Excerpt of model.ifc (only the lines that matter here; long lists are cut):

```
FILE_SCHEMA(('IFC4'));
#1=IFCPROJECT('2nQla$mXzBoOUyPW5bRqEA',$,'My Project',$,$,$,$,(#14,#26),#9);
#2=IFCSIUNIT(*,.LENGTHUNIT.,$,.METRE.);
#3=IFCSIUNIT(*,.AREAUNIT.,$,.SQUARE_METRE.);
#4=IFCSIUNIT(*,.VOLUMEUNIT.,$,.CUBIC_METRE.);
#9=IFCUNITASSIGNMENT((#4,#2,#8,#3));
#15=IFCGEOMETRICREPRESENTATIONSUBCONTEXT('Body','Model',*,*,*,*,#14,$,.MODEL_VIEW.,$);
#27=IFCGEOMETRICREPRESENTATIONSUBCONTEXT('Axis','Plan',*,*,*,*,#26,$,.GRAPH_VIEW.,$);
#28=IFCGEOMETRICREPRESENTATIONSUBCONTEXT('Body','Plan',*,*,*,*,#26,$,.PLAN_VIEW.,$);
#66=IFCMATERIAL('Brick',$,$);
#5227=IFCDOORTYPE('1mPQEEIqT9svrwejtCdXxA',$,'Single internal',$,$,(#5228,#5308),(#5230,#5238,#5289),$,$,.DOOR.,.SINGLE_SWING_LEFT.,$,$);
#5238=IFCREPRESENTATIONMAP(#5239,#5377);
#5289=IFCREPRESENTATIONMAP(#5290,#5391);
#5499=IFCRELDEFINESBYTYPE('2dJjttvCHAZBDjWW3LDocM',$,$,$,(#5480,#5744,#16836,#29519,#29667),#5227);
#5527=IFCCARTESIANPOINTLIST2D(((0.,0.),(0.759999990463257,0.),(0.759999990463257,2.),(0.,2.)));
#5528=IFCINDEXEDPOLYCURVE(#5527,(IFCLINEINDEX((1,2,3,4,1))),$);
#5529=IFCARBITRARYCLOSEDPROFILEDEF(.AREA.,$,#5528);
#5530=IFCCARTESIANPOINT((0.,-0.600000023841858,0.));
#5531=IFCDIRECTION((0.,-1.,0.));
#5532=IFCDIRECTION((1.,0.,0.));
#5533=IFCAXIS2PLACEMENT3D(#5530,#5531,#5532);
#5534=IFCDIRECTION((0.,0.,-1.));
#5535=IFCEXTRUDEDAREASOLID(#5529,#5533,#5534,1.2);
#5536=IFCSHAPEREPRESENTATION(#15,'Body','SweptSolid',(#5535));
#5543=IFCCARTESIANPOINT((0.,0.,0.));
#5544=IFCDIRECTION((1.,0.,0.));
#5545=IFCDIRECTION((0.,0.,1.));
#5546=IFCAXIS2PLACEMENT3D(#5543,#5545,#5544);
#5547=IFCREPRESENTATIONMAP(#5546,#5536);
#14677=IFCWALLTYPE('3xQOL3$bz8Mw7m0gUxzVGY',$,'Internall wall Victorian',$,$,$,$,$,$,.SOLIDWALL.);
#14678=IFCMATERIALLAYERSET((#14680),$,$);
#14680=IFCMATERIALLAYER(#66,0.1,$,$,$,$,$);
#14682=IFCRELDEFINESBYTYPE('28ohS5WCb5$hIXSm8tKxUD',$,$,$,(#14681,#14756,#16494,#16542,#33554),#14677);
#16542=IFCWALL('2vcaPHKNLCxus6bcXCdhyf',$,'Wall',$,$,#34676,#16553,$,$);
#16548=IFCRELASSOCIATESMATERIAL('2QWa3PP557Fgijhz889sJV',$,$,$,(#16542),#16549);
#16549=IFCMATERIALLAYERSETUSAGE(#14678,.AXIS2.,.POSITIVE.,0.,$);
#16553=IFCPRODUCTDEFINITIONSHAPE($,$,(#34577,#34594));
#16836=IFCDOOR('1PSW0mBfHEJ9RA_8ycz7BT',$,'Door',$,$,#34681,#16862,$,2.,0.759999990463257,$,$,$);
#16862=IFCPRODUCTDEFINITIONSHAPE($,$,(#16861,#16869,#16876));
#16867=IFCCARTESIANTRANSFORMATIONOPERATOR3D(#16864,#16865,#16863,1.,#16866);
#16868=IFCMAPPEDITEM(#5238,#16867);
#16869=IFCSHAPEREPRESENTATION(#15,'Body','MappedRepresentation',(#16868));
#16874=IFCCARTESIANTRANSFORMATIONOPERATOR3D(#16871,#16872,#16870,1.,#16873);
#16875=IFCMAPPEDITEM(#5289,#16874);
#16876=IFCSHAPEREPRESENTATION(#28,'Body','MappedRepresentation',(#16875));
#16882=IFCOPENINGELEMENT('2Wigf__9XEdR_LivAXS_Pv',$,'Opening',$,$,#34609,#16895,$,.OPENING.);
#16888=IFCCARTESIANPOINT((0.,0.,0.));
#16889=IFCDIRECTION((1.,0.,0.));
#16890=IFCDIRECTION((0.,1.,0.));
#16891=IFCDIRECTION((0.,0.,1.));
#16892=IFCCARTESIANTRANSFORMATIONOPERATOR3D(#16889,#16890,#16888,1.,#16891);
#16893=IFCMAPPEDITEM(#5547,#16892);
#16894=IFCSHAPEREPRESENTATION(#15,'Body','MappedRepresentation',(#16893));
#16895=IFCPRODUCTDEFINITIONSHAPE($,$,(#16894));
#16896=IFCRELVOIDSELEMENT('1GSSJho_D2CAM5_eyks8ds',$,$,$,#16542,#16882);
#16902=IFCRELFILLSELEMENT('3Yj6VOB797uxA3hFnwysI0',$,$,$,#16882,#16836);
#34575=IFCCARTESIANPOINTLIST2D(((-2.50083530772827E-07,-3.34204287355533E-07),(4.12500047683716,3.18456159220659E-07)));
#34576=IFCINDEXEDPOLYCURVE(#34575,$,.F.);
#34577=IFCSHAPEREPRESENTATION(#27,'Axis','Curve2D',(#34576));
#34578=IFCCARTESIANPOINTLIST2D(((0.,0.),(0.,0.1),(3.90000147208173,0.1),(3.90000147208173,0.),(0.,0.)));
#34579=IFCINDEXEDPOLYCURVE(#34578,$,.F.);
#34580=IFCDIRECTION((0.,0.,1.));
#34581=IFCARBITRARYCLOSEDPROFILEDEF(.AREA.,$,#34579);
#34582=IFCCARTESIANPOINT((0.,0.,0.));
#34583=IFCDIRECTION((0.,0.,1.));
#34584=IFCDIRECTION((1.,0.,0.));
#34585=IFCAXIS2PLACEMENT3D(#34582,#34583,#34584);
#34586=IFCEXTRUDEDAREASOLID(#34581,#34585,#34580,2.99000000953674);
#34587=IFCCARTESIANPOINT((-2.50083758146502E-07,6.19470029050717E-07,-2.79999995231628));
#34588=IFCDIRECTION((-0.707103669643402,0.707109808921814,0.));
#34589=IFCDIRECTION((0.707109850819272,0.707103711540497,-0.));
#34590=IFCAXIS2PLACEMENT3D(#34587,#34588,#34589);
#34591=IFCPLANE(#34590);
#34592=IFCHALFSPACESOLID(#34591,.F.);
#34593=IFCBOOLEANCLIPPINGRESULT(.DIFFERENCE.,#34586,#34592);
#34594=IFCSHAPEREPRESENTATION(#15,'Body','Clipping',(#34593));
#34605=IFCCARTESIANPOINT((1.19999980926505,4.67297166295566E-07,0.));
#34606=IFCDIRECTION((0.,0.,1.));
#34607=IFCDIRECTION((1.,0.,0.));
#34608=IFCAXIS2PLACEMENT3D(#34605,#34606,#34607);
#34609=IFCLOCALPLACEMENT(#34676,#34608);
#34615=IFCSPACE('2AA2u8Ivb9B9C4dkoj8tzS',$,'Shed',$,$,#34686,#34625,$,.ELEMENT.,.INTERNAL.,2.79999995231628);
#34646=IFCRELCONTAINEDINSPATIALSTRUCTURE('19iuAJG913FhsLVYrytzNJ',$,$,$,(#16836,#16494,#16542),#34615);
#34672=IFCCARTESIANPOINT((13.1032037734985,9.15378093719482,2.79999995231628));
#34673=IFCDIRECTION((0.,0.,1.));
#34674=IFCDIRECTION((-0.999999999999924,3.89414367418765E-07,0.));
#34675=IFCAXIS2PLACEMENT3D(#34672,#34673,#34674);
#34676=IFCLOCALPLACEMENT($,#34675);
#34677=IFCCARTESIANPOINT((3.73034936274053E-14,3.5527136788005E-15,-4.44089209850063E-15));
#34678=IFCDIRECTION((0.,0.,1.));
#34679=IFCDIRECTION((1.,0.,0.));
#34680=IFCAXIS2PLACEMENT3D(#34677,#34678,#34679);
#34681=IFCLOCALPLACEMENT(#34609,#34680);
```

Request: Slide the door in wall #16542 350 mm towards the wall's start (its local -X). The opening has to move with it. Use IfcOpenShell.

```python
import ifcopenshell
import ifcopenshell.api.geometry
import ifcopenshell.util.placement
import ifcopenshell.util.unit

model = ifcopenshell.open("model.ifc")
unit_scale = ifcopenshell.util.unit.calculate_unit_scale(model)

door = model.by_guid("1PSW0mBfHEJ9RA_8ycz7BT")
opening = door.FillsVoids[0].RelatingOpeningElement
wall = opening.VoidsElements[0].RelatingBuildingElement

wall_matrix = ifcopenshell.util.placement.get_local_placement(wall.ObjectPlacement)
shift = wall_matrix[:3, 0] * -0.35 / unit_scale
before = ifcopenshell.util.placement.get_local_placement(door.ObjectPlacement)[:3, 3].copy()

# The door is placed relative to its opening, so it follows when the opening moves.
matrix = ifcopenshell.util.placement.get_local_placement(opening.ObjectPlacement)
matrix[:3, 3] += shift
ifcopenshell.api.geometry.edit_object_placement(
    model, product=opening, matrix=matrix, is_si=False, should_transform_children=True
)

after = ifcopenshell.util.placement.get_local_placement(door.ObjectPlacement)[:3, 3]
print("door moved by", (after - before).round(3) + 0.0)

model.write("model-out.ifc")
```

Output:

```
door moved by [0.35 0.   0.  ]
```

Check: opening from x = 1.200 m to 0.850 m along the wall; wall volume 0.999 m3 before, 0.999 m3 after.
